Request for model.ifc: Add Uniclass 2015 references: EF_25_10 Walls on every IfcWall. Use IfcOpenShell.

First a look at what the model holds.

```python
import ifcopenshell

model = ifcopenshell.open("model.ifc")
print(model.schema)
print("classifications:", [c.Name for c in model.by_type("IfcClassification")])
for ifc_class in ("IfcDoor", "IfcRoof", "IfcStair", "IfcWall", "IfcWindow"):
    print(ifc_class, len(model.by_type(ifc_class)))
```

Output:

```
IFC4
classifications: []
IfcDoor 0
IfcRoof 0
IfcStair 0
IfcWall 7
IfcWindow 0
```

```python
import ifcopenshell
import ifcopenshell.api.classification

model = ifcopenshell.open("model.ifc")

system = ifcopenshell.api.classification.add_classification(model, classification="Uniclass 2015")

codes = {
    "IfcWall": ("EF_25_10", "Walls"),
}
for ifc_class, (code, name) in codes.items():
    products = model.by_type(ifc_class)
    ifcopenshell.api.classification.add_reference(
        model, products=products, classification=system, identification=code, name=name
    )
    print(code, len(products))

model.write("model_v2.ifc")
```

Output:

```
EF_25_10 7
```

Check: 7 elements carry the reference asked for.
